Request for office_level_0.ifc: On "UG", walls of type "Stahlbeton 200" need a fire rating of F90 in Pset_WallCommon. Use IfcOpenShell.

First a look at what the model holds.

```python
import ifcopenshell
import ifcopenshell.util.element

model = ifcopenshell.open("office_level_0.ifc")
print(model.schema)
storey = next(s for s in model.by_type("IfcBuildingStorey") if s.Name == "UG")
walls = [e for e in ifcopenshell.util.element.get_decomposition(storey) if e.is_a("IfcWall")]
seen = {}
for e in walls:
    element_type = ifcopenshell.util.element.get_type(e)
    key = (element_type.Name if element_type != e and element_type else None, ifcopenshell.util.element.get_pset(e, "Pset_WallCommon", "FireRating"))
    seen[key] = seen.get(key, 0) + 1
for (name, value), count in sorted(seen.items(), key=str):
    print(count, "x", name, "|", value)
```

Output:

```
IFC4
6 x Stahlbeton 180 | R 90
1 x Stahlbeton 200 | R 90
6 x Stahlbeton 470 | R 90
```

```python
import ifcopenshell
import ifcopenshell.api.pset
import ifcopenshell.util.element

model = ifcopenshell.open("office_level_0.ifc")

storey = next(s for s in model.by_type("IfcBuildingStorey") if s.Name == "UG")
walls = [e for e in ifcopenshell.util.element.get_decomposition(storey) if e.is_a("IfcWall")]

count = 0
for e in walls:
    element_type = ifcopenshell.util.element.get_type(e)
    if element_type in (None, e) or element_type.Name != "Stahlbeton 200":
        continue
    # add_pset returns the element's existing set when there is one.
    pset = ifcopenshell.api.pset.add_pset(model, product=e, name="Pset_WallCommon")
    ifcopenshell.api.pset.edit_pset(model, pset=pset, properties={"FireRating": "F90"})
    count += 1

print(count, "walls updated")

model.write("office_level_0_updated.ifc")
```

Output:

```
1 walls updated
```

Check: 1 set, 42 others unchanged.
